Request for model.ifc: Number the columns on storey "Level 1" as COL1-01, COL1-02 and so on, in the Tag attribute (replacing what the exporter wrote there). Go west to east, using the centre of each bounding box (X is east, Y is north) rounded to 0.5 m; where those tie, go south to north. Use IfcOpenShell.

First a look at what the model holds.

```python
import ifcopenshell
import ifcopenshell.util.element
import ifcopenshell.util.placement

model = ifcopenshell.open("model.ifc")
print(model.schema)
storey = next(s for s in model.by_type("IfcBuildingStorey") if s.Name == "Level 1")
columns = [e for e in ifcopenshell.util.element.get_decomposition(storey) if e.is_a("IfcColumn")]
for e in sorted(columns, key=lambda e: e.id()):
    origin = ifcopenshell.util.placement.get_local_placement(e.ObjectPlacement)[:3, 3]
    print(e.id(), e.Tag, e.Name, origin.round(2) + 0.0, sep=" | ")
```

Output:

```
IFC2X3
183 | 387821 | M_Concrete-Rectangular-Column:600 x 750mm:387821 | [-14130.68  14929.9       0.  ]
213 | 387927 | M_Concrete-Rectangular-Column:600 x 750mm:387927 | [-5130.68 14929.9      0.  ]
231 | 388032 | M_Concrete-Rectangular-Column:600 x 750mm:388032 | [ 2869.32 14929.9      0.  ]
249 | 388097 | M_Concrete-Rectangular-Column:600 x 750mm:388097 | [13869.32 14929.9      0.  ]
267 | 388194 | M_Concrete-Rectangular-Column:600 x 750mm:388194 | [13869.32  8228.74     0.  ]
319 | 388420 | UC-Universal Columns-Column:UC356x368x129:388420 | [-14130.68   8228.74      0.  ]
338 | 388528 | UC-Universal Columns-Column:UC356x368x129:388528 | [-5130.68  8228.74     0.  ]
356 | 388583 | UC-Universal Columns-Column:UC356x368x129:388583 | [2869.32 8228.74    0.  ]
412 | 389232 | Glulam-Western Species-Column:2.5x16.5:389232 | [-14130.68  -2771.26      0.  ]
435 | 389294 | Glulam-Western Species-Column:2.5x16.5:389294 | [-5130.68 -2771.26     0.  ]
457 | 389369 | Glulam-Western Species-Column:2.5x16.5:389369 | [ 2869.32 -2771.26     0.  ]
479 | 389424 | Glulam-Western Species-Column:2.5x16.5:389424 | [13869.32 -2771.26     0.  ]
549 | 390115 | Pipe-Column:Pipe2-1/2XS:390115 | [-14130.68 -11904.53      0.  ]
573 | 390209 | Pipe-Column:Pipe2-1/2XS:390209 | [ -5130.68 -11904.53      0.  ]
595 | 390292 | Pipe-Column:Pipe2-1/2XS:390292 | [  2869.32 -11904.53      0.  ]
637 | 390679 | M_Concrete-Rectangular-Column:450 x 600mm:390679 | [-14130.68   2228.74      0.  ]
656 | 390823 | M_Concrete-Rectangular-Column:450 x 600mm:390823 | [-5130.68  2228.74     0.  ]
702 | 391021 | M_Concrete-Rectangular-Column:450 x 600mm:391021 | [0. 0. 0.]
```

```python
import ifcopenshell
import ifcopenshell.geom
import ifcopenshell.util.element
import ifcopenshell.util.shape

model = ifcopenshell.open("model.ifc")
settings = ifcopenshell.geom.settings()
settings.set("use-world-coords", True)


def centre(element):
    shape = ifcopenshell.geom.create_shape(settings, element)
    return ifcopenshell.util.shape.get_bbox_centroid(shape.geometry)


storey = next(s for s in model.by_type("IfcBuildingStorey") if s.Name == "Level 1")
columns = [e for e in ifcopenshell.util.element.get_decomposition(storey) if e.is_a("IfcColumn")]

# Insertion points can sit at a corner or the storey origin, so sort by the geometry (in metres).
centres = {e: centre(e) for e in columns}
columns.sort(key=lambda e: (round(centres[e][0] / 0.5), centres[e][1]))

for i, e in enumerate(columns, start=1):
    number = f"COL1-{i:02d}"
    e.Tag = number
    print(e.id(), number)

model.write("model_edited.ifc")
```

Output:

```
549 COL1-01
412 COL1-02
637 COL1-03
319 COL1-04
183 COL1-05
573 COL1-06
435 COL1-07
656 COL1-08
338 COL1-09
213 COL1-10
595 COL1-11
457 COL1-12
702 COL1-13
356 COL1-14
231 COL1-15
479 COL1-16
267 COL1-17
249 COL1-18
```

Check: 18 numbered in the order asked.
